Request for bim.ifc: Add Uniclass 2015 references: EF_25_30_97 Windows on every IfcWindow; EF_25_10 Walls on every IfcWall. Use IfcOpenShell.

First a look at what the model holds.

```python
import ifcopenshell

model = ifcopenshell.open("bim.ifc")
print(model.schema)
print("classifications:", [c.Name for c in model.by_type("IfcClassification")])
for ifc_class in ("IfcDoor", "IfcRoof", "IfcStair", "IfcWall", "IfcWindow"):
    print(ifc_class, len(model.by_type(ifc_class)))
```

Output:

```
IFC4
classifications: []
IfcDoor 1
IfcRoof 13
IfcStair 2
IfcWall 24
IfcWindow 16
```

```python
import ifcopenshell
import ifcopenshell.api.classification

model = ifcopenshell.open("bim.ifc")

system = ifcopenshell.api.classification.add_classification(model, classification="Uniclass 2015")

codes = {
    "IfcWindow": ("EF_25_30_97", "Windows"),
    "IfcWall": ("EF_25_10", "Walls"),
}
for ifc_class, (code, name) in codes.items():
    products = model.by_type(ifc_class)
    ifcopenshell.api.classification.add_reference(
        model, products=products, classification=system, identification=code, name=name
    )
    print(code, len(products))

model.write("bim_v2.ifc")
```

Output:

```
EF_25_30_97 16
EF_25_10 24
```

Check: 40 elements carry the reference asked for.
